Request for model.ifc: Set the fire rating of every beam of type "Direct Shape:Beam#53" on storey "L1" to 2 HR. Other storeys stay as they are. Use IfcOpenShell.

First a look at what the model holds.

```python
import ifcopenshell
import ifcopenshell.util.element

model = ifcopenshell.open("model.ifc")
print(model.schema)
storey = next(s for s in model.by_type("IfcBuildingStorey") if s.Name == "L1")
beams = [e for e in ifcopenshell.util.element.get_decomposition(storey) if e.is_a("IfcBeam")]
seen = {}
for e in beams:
    element_type = ifcopenshell.util.element.get_type(e)
    key = (element_type.Name if element_type != e and element_type else None, ifcopenshell.util.element.get_pset(e, "Pset_BeamCommon", "FireRating"))
    seen[key] = seen.get(key, 0) + 1
for (name, value), count in sorted(seen.items(), key=str):
    print(count, "x", name, "|", value)
```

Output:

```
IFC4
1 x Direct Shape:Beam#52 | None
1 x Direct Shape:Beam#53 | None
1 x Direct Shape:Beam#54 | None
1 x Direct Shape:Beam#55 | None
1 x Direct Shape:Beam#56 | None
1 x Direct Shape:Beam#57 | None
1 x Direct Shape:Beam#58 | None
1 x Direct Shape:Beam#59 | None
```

```python
import ifcopenshell
import ifcopenshell.api.pset
import ifcopenshell.util.element

model = ifcopenshell.open("model.ifc")

storey = next(s for s in model.by_type("IfcBuildingStorey") if s.Name == "L1")
beams = [e for e in ifcopenshell.util.element.get_decomposition(storey) if e.is_a("IfcBeam")]

count = 0
for e in beams:
    element_type = ifcopenshell.util.element.get_type(e)
    if element_type in (None, e) or element_type.Name != "Direct Shape:Beam#53":
        continue
    # add_pset returns the element's existing set when there is one.
    pset = ifcopenshell.api.pset.add_pset(model, product=e, name="Pset_BeamCommon")
    ifcopenshell.api.pset.edit_pset(model, pset=pset, properties={"FireRating": "2 HR"})
    count += 1

print(count, "beams updated")

model.write("model_rev.ifc")
```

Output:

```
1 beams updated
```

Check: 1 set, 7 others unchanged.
